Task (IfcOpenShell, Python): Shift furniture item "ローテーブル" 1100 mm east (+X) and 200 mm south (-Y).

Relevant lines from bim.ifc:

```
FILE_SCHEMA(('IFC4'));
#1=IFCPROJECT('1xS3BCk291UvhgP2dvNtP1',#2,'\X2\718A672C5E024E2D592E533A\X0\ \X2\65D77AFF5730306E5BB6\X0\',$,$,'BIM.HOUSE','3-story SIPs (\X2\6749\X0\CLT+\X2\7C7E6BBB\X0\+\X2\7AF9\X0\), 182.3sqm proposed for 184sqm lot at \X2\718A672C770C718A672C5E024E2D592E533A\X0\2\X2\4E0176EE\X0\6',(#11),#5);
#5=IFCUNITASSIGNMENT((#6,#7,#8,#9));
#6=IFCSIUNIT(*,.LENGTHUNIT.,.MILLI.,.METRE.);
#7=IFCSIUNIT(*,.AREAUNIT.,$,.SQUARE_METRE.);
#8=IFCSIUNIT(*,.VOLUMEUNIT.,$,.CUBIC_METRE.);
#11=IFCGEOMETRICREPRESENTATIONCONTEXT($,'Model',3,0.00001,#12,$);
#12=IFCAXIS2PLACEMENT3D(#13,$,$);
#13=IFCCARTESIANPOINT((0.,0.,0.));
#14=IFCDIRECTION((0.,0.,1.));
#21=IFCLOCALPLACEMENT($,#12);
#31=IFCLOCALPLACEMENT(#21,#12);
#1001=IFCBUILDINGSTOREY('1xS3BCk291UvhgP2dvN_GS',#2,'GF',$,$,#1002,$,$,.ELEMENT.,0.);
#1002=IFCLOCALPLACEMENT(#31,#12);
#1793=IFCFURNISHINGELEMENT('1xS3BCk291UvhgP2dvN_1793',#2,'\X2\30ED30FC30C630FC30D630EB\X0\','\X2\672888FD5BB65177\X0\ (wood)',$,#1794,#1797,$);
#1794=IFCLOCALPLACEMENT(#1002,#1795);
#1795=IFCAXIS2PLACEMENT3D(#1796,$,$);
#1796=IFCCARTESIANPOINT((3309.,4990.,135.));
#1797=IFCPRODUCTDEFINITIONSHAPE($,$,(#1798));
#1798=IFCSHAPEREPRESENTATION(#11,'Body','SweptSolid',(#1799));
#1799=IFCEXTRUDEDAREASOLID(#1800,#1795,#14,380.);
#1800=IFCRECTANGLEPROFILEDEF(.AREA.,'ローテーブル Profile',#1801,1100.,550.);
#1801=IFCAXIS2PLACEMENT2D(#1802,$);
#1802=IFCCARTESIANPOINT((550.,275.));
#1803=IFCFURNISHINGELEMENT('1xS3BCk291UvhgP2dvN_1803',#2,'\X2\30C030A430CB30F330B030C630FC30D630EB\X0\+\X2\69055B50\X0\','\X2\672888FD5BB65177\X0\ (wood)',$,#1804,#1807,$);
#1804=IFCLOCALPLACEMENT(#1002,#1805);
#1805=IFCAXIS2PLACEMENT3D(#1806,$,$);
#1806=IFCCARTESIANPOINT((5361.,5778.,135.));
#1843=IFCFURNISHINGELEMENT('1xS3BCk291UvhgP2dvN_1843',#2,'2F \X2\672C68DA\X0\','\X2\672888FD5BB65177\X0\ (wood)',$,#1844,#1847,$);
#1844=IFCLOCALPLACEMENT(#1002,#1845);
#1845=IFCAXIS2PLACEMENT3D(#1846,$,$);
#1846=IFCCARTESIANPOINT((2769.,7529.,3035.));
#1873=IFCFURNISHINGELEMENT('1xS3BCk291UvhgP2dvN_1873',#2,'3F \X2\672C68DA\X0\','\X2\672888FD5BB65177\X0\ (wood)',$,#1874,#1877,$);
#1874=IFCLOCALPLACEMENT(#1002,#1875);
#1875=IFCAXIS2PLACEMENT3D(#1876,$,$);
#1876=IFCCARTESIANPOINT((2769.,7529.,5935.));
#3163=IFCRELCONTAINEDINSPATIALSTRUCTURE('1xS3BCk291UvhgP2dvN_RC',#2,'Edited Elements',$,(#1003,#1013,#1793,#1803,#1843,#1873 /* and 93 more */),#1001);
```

```python
import ifcopenshell
import ifcopenshell.api.geometry
import ifcopenshell.util.placement
import ifcopenshell.util.unit

model = ifcopenshell.open("bim.ifc")
unit_scale = ifcopenshell.util.unit.calculate_unit_scale(model)

item = model.by_guid("1xS3BCk291UvhgP2dvN_1793")
matrix = ifcopenshell.util.placement.get_local_placement(item.ObjectPlacement)
matrix[0, 3] += 1.1 / unit_scale
matrix[1, 3] -= 0.2 / unit_scale
ifcopenshell.api.geometry.edit_object_placement(model, product=item, matrix=matrix, is_si=False)

print(ifcopenshell.util.placement.get_local_placement(item.ObjectPlacement).round(3) + 0.0)

model.write("bim_edited.ifc")
```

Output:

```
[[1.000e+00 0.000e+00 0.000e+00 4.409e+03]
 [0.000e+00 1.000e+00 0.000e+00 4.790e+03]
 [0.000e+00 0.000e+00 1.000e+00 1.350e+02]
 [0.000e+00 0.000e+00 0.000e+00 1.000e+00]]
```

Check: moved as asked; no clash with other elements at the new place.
